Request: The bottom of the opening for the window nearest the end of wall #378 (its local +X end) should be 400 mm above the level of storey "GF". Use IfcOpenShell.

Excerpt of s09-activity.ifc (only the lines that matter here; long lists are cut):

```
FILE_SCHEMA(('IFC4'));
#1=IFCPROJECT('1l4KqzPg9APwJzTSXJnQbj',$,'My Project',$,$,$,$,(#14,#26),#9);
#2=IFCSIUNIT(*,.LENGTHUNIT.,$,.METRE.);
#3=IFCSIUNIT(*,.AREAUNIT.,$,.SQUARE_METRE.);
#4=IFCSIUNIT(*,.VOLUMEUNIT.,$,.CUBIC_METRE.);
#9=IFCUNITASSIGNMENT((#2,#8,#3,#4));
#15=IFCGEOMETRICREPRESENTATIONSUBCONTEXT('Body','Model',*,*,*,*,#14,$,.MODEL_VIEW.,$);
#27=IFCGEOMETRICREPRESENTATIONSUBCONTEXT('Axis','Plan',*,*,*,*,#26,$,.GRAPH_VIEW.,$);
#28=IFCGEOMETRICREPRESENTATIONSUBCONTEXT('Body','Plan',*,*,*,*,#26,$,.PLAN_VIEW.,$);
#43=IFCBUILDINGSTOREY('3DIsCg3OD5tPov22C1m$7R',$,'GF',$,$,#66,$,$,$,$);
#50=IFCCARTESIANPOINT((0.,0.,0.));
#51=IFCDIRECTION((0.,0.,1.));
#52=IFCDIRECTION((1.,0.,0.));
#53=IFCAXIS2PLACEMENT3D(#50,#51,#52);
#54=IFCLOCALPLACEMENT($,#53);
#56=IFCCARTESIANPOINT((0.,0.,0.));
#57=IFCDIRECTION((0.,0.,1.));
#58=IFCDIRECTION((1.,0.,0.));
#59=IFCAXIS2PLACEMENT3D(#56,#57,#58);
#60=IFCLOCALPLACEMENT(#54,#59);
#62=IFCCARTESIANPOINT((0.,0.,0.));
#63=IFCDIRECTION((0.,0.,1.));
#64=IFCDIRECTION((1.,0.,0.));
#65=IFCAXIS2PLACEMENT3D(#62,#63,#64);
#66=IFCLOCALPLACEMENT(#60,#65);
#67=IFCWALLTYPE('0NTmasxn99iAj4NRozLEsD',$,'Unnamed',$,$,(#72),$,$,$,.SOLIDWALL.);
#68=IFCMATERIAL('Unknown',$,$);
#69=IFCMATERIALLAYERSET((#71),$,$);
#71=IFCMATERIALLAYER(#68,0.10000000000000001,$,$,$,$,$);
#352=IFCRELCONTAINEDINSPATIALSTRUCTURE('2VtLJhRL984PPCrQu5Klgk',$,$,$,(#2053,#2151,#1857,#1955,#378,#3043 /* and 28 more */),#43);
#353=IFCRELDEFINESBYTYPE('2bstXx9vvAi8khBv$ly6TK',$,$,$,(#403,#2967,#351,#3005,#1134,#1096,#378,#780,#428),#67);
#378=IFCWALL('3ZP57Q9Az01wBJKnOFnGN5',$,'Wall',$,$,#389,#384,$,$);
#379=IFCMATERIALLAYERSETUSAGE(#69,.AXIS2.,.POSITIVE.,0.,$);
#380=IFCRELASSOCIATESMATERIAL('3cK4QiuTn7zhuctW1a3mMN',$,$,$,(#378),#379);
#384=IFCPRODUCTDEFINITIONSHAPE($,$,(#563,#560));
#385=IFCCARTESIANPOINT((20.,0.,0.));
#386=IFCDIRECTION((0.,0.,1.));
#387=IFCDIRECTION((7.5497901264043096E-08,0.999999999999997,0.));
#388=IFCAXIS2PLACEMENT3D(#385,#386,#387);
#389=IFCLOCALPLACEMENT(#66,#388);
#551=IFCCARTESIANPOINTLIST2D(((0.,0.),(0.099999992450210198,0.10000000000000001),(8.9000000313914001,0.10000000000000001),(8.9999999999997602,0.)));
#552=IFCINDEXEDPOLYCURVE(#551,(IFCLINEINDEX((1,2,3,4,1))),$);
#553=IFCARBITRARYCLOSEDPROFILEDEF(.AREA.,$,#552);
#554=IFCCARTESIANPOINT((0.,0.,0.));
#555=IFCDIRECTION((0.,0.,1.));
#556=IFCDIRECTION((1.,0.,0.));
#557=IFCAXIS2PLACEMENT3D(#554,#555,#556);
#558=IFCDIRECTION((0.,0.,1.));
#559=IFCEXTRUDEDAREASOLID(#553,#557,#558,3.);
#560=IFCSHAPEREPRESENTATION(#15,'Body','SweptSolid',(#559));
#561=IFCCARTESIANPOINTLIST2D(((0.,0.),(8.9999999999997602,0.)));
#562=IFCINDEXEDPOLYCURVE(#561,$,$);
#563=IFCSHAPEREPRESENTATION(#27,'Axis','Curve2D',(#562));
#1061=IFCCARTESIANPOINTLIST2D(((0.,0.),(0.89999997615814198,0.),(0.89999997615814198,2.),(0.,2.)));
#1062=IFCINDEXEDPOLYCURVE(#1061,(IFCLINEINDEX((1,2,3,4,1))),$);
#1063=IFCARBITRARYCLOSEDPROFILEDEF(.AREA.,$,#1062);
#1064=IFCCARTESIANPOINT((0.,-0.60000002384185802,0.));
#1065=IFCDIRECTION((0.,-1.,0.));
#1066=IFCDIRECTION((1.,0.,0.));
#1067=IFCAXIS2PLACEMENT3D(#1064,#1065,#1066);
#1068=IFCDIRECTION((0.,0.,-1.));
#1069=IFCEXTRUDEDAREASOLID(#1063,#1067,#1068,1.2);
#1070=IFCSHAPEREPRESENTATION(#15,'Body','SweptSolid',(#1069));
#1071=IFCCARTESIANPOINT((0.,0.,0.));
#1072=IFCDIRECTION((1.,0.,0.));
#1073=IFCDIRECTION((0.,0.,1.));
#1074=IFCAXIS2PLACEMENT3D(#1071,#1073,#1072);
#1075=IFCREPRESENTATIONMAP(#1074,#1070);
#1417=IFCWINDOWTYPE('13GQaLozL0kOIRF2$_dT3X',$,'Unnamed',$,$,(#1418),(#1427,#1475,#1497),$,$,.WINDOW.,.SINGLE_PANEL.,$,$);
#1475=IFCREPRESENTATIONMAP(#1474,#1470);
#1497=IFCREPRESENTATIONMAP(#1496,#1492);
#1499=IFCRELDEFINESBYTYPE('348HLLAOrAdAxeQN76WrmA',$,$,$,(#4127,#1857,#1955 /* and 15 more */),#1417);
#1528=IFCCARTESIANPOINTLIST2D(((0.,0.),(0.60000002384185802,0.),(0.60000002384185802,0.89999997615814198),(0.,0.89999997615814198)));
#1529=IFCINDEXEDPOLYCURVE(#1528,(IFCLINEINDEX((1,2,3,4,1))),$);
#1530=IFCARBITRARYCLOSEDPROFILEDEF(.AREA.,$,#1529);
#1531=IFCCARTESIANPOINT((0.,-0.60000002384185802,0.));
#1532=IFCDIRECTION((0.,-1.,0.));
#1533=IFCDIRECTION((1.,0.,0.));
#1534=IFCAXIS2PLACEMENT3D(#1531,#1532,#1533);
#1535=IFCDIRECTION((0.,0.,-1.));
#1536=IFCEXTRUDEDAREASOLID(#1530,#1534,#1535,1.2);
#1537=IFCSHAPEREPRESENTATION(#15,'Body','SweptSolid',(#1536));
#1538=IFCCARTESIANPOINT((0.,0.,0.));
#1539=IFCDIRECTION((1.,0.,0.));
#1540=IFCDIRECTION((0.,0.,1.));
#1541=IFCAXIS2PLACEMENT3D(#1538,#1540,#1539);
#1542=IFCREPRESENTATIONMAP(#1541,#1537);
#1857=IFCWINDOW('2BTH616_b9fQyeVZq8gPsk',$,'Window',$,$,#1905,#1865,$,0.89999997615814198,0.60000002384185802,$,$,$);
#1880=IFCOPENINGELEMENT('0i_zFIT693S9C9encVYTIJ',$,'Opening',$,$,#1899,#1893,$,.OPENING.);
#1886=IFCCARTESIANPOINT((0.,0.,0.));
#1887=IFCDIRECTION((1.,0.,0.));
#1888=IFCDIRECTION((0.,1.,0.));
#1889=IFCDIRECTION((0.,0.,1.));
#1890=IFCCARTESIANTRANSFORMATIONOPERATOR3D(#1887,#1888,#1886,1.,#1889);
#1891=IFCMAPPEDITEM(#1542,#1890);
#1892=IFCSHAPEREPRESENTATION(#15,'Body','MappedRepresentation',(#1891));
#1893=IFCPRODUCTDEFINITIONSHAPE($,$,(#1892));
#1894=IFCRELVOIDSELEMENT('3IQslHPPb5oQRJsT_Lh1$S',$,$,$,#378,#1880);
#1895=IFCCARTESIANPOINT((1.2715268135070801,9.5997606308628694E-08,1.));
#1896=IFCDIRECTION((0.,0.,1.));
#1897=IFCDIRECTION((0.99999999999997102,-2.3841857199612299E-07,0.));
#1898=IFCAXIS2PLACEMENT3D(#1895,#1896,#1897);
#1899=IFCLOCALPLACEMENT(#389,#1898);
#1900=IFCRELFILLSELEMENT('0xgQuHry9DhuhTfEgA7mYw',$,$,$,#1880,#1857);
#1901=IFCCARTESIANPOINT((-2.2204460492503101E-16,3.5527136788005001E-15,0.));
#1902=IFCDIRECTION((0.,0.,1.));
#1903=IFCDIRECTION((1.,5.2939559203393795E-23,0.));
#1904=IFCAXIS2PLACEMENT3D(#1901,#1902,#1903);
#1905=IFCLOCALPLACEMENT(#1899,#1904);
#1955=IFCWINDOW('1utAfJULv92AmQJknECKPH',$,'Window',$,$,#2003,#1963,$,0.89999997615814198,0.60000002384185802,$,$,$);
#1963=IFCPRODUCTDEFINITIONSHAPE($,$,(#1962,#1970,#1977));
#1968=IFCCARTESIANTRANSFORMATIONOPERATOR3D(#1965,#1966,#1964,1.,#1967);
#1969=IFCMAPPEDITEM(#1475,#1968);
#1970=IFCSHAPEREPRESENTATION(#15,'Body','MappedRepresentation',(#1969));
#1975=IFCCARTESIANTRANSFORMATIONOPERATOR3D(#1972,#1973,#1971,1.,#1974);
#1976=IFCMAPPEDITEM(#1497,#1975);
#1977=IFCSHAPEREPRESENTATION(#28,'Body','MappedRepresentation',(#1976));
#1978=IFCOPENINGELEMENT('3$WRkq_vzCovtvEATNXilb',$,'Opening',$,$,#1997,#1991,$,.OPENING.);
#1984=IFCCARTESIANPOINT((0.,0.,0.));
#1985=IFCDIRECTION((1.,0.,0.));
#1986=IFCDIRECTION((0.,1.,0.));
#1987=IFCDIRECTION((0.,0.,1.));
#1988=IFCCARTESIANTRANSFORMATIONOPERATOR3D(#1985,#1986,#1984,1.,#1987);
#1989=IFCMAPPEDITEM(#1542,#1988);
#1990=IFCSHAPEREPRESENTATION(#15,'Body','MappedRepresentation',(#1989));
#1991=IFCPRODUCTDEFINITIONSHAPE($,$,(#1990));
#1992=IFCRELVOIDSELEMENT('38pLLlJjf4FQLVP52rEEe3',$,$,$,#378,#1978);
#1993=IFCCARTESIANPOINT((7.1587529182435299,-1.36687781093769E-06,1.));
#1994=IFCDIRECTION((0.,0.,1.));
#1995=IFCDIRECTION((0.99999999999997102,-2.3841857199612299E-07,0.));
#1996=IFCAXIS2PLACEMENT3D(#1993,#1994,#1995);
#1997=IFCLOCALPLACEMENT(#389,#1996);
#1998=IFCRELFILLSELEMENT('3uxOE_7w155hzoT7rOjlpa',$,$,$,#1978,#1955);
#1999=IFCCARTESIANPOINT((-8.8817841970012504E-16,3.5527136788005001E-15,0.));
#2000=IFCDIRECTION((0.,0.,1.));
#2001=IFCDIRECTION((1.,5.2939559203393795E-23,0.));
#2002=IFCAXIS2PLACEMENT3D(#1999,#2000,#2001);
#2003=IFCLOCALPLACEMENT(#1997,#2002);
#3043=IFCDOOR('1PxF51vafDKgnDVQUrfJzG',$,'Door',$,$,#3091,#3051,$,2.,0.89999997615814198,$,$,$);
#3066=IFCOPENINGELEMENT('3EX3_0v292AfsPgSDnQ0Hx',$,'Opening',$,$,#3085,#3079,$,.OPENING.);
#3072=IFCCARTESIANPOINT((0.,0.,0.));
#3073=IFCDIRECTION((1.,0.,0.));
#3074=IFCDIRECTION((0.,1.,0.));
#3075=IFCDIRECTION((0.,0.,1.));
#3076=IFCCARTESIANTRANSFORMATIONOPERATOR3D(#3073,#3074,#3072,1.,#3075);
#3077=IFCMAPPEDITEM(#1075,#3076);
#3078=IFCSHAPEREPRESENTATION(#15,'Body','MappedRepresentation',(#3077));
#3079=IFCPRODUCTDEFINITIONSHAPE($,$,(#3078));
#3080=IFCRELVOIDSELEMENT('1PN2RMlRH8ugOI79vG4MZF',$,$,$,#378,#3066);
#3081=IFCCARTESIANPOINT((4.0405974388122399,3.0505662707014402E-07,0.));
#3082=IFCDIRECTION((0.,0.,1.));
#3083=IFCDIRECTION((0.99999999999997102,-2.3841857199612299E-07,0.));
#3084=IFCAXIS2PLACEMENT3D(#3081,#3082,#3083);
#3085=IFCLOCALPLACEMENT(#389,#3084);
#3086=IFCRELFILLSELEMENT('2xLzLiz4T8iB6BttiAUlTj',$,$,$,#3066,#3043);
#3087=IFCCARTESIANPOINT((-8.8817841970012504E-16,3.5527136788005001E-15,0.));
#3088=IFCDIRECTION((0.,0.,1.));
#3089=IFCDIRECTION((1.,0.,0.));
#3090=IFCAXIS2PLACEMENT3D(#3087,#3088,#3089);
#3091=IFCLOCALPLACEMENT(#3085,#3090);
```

```python
import numpy as np
import ifcopenshell
import ifcopenshell.api.geometry
import ifcopenshell.geom
import ifcopenshell.util.element
import ifcopenshell.util.placement
import ifcopenshell.util.shape
import ifcopenshell.util.unit

model = ifcopenshell.open("s09-activity.ifc")
unit_scale = ifcopenshell.util.unit.calculate_unit_scale(model)

window = model.by_guid("1utAfJULv92AmQJknECKPH")
opening = window.FillsVoids[0].RelatingOpeningElement
storey = ifcopenshell.util.element.get_container(window, ifc_class="IfcBuildingStorey")
level = ifcopenshell.util.placement.get_local_placement(storey.ObjectPlacement)[2, 3]

# The opening's origin need not be at the sill, so measure its lowest point.
shape = ifcopenshell.geom.create_shape(ifcopenshell.geom.settings(), opening)
bottom = ifcopenshell.util.shape.get_shape_bottom_elevation(shape, shape.geometry) / unit_scale
dz = level + 0.4 - bottom

shift = np.array([0.0, 0.0, dz])
# The window is placed relative to its opening, so it follows when the opening moves.
matrix = ifcopenshell.util.placement.get_local_placement(opening.ObjectPlacement)
matrix[:3, 3] += shift
ifcopenshell.api.geometry.edit_object_placement(
    model, product=opening, matrix=matrix, is_si=False, should_transform_children=True
)

print(f"moved by {dz * unit_scale:+.3f} m")

model.write("s09-activity_edited.ifc")
```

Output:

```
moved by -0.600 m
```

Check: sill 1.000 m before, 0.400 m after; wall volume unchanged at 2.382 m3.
